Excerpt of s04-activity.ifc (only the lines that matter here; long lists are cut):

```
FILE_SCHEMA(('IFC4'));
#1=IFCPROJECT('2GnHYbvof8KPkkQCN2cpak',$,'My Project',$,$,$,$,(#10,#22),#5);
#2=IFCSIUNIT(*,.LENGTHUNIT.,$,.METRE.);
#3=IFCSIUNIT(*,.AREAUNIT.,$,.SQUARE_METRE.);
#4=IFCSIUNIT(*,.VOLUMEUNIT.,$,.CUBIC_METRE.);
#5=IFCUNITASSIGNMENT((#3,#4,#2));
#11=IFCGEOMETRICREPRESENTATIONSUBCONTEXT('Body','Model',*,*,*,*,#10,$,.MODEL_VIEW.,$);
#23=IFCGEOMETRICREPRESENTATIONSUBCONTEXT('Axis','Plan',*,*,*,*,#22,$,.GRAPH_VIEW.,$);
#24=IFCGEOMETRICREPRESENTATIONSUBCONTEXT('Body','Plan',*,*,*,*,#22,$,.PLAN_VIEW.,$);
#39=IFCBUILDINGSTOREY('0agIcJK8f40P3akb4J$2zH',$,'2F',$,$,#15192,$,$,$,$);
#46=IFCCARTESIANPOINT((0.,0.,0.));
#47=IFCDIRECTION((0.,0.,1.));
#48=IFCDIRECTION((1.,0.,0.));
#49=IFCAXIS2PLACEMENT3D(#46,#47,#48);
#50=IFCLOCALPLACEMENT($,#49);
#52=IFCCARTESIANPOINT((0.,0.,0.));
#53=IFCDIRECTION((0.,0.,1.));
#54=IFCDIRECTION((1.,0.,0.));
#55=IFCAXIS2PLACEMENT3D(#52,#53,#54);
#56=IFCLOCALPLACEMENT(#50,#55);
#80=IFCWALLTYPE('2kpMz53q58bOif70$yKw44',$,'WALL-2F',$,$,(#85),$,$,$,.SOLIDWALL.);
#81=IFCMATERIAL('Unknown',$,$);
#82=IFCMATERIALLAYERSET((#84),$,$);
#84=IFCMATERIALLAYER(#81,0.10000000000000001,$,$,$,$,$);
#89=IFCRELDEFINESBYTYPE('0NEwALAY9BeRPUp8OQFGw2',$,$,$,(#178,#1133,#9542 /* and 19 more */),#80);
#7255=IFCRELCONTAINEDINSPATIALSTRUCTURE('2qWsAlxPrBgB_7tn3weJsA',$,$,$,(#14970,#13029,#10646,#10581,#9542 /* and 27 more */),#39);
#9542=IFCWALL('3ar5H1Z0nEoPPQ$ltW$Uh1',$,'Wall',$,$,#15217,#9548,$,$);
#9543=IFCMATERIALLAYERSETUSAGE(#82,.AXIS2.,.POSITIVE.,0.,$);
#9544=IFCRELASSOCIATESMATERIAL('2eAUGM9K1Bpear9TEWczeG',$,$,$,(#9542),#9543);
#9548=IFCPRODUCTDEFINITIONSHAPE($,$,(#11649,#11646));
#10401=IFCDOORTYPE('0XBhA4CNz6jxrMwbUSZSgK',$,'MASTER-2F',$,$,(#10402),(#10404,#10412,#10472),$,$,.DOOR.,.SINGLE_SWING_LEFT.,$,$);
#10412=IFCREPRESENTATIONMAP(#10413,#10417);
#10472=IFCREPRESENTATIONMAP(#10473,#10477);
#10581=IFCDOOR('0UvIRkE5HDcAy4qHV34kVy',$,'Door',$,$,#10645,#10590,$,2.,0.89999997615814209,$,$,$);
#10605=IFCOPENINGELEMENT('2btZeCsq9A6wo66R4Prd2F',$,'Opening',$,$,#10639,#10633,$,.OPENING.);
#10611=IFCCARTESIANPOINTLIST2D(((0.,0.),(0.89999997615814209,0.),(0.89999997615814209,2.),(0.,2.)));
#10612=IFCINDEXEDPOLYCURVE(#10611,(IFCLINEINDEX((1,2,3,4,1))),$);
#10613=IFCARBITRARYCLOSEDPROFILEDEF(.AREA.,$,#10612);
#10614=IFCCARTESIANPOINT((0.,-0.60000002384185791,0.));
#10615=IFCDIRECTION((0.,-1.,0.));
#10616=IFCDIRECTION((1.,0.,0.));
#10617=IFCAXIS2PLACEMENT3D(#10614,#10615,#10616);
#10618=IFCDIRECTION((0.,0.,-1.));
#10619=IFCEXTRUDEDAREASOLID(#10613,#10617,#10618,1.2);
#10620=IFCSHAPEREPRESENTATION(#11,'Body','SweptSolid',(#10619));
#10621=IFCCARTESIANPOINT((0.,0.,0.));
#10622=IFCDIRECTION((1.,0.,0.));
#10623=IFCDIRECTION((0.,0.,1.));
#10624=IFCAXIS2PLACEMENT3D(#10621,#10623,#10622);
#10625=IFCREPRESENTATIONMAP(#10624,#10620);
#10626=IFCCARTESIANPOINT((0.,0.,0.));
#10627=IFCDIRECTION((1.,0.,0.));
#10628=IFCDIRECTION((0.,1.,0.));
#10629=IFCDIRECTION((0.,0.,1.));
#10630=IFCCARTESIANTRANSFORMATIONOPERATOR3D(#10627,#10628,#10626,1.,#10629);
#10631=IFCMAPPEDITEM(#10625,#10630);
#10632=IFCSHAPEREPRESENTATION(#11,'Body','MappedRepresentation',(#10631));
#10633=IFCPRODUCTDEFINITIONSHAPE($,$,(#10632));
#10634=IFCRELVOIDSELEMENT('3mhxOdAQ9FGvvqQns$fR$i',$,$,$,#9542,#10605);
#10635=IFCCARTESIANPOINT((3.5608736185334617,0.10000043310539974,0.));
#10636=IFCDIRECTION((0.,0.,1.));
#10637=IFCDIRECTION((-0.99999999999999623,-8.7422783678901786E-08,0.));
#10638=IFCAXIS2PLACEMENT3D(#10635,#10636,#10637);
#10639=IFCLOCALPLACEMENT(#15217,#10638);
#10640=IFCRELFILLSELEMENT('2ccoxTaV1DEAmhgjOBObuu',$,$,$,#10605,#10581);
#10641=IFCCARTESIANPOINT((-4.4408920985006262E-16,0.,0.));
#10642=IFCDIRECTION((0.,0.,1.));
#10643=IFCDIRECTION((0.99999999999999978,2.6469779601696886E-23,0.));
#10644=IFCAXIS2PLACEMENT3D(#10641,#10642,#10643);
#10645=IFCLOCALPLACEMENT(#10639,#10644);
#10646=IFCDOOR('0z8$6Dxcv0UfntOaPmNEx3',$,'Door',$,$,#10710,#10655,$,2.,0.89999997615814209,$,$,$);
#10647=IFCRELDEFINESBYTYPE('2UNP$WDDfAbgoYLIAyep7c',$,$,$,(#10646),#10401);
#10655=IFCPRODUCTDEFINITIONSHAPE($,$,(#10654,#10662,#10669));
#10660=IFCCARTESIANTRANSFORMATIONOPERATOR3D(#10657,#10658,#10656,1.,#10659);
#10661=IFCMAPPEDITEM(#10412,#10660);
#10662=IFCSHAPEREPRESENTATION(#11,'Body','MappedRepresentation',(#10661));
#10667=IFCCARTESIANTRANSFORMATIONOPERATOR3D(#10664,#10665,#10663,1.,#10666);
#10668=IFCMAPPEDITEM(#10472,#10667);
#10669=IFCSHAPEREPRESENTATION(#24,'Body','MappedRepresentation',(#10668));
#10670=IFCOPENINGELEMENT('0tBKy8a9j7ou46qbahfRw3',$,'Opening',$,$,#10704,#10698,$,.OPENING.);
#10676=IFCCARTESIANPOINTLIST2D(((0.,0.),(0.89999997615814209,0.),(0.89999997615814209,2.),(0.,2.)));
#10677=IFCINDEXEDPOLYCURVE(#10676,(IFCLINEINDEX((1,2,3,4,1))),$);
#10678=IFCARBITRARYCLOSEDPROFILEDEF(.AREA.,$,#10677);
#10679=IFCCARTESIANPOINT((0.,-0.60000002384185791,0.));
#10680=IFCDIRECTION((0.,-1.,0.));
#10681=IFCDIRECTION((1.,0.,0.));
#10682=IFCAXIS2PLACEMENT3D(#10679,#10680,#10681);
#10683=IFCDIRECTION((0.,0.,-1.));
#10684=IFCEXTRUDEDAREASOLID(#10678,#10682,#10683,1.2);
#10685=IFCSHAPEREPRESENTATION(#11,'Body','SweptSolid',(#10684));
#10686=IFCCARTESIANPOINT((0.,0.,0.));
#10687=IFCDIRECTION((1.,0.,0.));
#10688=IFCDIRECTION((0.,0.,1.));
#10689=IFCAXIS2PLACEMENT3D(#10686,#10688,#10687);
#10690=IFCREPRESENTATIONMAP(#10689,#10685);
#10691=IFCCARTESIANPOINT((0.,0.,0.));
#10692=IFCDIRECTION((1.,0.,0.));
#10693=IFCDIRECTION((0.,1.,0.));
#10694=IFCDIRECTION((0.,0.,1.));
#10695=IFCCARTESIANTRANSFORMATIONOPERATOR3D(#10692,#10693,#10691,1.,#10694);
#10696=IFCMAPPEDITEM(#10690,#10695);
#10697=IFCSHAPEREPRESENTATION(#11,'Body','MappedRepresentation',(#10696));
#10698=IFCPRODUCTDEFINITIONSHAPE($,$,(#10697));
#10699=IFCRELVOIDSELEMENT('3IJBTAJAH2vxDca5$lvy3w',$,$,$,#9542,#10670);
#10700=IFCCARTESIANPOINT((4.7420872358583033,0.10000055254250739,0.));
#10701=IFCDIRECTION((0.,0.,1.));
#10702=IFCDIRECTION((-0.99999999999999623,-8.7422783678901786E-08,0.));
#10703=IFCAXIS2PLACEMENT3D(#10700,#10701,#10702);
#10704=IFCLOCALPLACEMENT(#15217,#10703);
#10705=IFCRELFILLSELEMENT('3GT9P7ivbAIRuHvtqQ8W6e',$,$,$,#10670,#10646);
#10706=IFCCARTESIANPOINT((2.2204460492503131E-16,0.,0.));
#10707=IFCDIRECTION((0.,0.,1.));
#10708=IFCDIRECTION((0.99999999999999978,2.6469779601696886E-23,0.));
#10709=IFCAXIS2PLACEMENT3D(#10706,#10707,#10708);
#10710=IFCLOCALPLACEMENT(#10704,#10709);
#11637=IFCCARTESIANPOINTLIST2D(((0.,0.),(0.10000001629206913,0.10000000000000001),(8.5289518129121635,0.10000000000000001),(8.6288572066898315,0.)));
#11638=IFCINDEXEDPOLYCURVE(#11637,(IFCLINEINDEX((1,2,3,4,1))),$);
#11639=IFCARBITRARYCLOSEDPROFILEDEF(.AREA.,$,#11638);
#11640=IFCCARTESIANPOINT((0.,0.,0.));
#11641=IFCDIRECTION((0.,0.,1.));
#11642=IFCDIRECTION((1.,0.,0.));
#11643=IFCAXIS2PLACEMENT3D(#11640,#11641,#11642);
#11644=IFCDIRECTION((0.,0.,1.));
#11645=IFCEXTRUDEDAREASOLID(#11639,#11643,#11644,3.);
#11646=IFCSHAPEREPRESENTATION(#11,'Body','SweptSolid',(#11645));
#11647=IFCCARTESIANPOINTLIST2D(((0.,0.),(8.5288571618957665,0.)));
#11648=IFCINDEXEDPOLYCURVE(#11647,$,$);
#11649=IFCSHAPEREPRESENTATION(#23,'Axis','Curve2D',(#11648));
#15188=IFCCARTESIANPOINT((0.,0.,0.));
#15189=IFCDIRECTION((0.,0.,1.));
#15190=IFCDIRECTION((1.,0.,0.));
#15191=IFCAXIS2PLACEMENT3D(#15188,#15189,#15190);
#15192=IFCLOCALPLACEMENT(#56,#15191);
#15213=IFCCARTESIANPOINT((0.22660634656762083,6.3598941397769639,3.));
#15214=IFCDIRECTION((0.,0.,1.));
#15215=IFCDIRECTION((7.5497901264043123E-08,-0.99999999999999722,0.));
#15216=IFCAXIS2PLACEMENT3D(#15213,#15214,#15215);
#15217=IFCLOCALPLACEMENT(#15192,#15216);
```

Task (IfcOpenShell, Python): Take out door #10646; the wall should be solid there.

```python
import ifcopenshell
import ifcopenshell.api.feature
import ifcopenshell.api.root
import ifcopenshell.geom
import ifcopenshell.util.shape

model = ifcopenshell.open("s04-activity.ifc")
settings = ifcopenshell.geom.settings()


def volume(element):
    """Net volume in cubic metres, openings subtracted."""
    shape = ifcopenshell.geom.create_shape(settings, element)
    return ifcopenshell.util.shape.get_volume(shape.geometry)


door = model.by_id(10646)
opening = door.FillsVoids[0].RelatingOpeningElement
wall = opening.VoidsElements[0].RelatingBuildingElement
before = volume(wall)

ifcopenshell.api.root.remove_product(model, product=door)
ifcopenshell.api.feature.remove_feature(model, feature=opening)

after = volume(wall)

print(f"wall volume {before:.3f} -> {after:.3f} m3")

model.write("s04-activity_v2.ifc")
```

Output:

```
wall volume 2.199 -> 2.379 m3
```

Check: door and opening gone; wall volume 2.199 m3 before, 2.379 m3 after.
